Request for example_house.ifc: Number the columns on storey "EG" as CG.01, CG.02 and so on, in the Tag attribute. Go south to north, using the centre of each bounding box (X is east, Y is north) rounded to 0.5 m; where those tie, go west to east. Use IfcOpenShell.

First a look at what the model holds.

```python
import ifcopenshell
import ifcopenshell.util.element
import ifcopenshell.util.placement

model = ifcopenshell.open("example_house.ifc")
print(model.schema)
storey = next(s for s in model.by_type("IfcBuildingStorey") if s.Name == "EG")
columns = [e for e in ifcopenshell.util.element.get_decomposition(storey) if e.is_a("IfcColumn")]
for e in sorted(columns, key=lambda e: e.id()):
    origin = ifcopenshell.util.placement.get_local_placement(e.ObjectPlacement)[:3, 3]
    print(e.id(), e.Tag, e.Name, origin.round(2) + 0.0, sep=" | ")
```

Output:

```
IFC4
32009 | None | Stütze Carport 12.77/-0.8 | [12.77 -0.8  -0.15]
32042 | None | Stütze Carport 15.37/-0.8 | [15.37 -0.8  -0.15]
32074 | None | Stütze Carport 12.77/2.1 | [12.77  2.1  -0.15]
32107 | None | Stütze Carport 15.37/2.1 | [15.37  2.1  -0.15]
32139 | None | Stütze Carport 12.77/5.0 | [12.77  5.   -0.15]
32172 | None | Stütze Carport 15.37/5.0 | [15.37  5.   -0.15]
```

```python
import ifcopenshell
import ifcopenshell.geom
import ifcopenshell.util.element
import ifcopenshell.util.shape

model = ifcopenshell.open("example_house.ifc")
settings = ifcopenshell.geom.settings()
settings.set("use-world-coords", True)


def centre(element):
    shape = ifcopenshell.geom.create_shape(settings, element)
    return ifcopenshell.util.shape.get_bbox_centroid(shape.geometry)


storey = next(s for s in model.by_type("IfcBuildingStorey") if s.Name == "EG")
columns = [e for e in ifcopenshell.util.element.get_decomposition(storey) if e.is_a("IfcColumn")]

# Insertion points can sit at a corner or the storey origin, so sort by the geometry (in metres).
centres = {e: centre(e) for e in columns}
columns.sort(key=lambda e: (round(centres[e][1] / 0.5), centres[e][0]))

for i, e in enumerate(columns, start=1):
    number = f"CG.{i:02d}"
    e.Tag = number
    print(e.id(), number)

model.write("example_house_v2.ifc")
```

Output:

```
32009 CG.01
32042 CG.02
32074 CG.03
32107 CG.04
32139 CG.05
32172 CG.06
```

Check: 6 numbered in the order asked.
